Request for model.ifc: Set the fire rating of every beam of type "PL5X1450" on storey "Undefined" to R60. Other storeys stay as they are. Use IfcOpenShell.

First a look at what the model holds.

```python
import ifcopenshell
import ifcopenshell.util.element

model = ifcopenshell.open("model.ifc")
print(model.schema)
storey = next(s for s in model.by_type("IfcBuildingStorey") if s.Name == "Undefined")
beams = [e for e in ifcopenshell.util.element.get_decomposition(storey) if e.is_a("IfcBeam")]
seen = {}
for e in beams:
    element_type = ifcopenshell.util.element.get_type(e)
    key = (element_type.Name if element_type != e and element_type else None, ifcopenshell.util.element.get_pset(e, "Pset_BeamCommon", "FireRating"))
    seen[key] = seen.get(key, 0) + 1
for (name, value), count in sorted(seen.items(), key=str):
    print(count, "x", name, "|", value)
```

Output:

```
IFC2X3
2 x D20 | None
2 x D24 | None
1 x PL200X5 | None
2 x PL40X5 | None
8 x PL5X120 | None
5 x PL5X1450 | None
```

```python
import ifcopenshell
import ifcopenshell.api.pset
import ifcopenshell.util.element

model = ifcopenshell.open("model.ifc")

storey = next(s for s in model.by_type("IfcBuildingStorey") if s.Name == "Undefined")
beams = [e for e in ifcopenshell.util.element.get_decomposition(storey) if e.is_a("IfcBeam")]

count = 0
for e in beams:
    element_type = ifcopenshell.util.element.get_type(e)
    if element_type in (None, e) or element_type.Name != "PL5X1450":
        continue
    # add_pset returns the element's existing set when there is one.
    pset = ifcopenshell.api.pset.add_pset(model, product=e, name="Pset_BeamCommon")
    ifcopenshell.api.pset.edit_pset(model, pset=pset, properties={"FireRating": "R60"})
    count += 1

print(count, "beams updated")

model.write("model_rev.ifc")
```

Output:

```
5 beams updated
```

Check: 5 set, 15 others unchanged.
